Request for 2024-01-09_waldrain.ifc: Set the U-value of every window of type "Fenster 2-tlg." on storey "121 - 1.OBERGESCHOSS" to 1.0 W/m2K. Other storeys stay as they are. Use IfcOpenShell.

First a look at what the model holds.

```python
import ifcopenshell
import ifcopenshell.util.element

model = ifcopenshell.open("2024-01-09_waldrain.ifc")
print(model.schema)
storey = next(s for s in model.by_type("IfcBuildingStorey") if s.Name == "121 - 1.OBERGESCHOSS")
windows = [e for e in ifcopenshell.util.element.get_decomposition(storey) if e.is_a("IfcWindow")]
seen = {}
for e in windows:
    element_type = ifcopenshell.util.element.get_type(e)
    key = (element_type.Name if element_type != e and element_type else None, ifcopenshell.util.element.get_pset(e, "Pset_WindowCommon", "ThermalTransmittance"))
    seen[key] = seen.get(key, 0) + 1
for (name, value), count in sorted(seen.items(), key=str):
    print(count, "x", name, "|", value)
```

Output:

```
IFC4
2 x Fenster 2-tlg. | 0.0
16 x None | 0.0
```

```python
import ifcopenshell
import ifcopenshell.api.pset
import ifcopenshell.util.element

model = ifcopenshell.open("2024-01-09_waldrain.ifc")

storey = next(s for s in model.by_type("IfcBuildingStorey") if s.Name == "121 - 1.OBERGESCHOSS")
windows = [e for e in ifcopenshell.util.element.get_decomposition(storey) if e.is_a("IfcWindow")]

count = 0
for e in windows:
    element_type = ifcopenshell.util.element.get_type(e)
    if element_type in (None, e) or element_type.Name != "Fenster 2-tlg.":
        continue
    # add_pset returns the element's existing set when there is one.
    pset = ifcopenshell.api.pset.add_pset(model, product=e, name="Pset_WindowCommon")
    ifcopenshell.api.pset.edit_pset(model, pset=pset, properties={"ThermalTransmittance": 1.0})
    count += 1

print(count, "windows updated")

model.write("2024-01-09_waldrain_updated.ifc")
```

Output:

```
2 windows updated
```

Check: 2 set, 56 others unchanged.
